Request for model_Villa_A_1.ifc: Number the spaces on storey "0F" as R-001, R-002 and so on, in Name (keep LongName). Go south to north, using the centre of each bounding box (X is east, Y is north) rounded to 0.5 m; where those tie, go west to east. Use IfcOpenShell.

First a look at what the model holds.

```python
import ifcopenshell
import ifcopenshell.util.element
import ifcopenshell.util.placement

model = ifcopenshell.open("model_Villa_A_1.ifc")
print(model.schema)
storey = next(s for s in model.by_type("IfcBuildingStorey") if s.Name == "0F")
spaces = [e for e in ifcopenshell.util.element.get_decomposition(storey) if e.is_a("IfcSpace")]
for e in sorted(spaces, key=lambda e: e.id()):
    origin = ifcopenshell.util.placement.get_local_placement(e.ObjectPlacement)[:3, 3]
    print(e.id(), e.Name, e.LongName, origin.round(2) + 0.0, sep=" | ")
```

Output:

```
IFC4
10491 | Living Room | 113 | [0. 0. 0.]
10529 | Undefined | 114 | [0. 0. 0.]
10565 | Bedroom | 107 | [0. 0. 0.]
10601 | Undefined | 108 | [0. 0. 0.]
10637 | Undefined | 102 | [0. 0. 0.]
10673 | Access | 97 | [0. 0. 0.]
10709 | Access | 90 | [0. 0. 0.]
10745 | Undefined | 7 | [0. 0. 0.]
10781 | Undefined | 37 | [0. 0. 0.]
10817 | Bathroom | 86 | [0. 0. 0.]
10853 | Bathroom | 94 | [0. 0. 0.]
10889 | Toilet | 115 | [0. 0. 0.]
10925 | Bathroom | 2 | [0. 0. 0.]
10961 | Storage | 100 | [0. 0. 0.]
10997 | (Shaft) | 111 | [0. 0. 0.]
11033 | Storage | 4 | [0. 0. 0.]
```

```python
import ifcopenshell
import ifcopenshell.geom
import ifcopenshell.util.element
import ifcopenshell.util.shape

model = ifcopenshell.open("model_Villa_A_1.ifc")
settings = ifcopenshell.geom.settings()
settings.set("use-world-coords", True)


def centre(element):
    shape = ifcopenshell.geom.create_shape(settings, element)
    return ifcopenshell.util.shape.get_bbox_centroid(shape.geometry)


storey = next(s for s in model.by_type("IfcBuildingStorey") if s.Name == "0F")
spaces = [e for e in ifcopenshell.util.element.get_decomposition(storey) if e.is_a("IfcSpace")]

# Insertion points can sit at a corner or the storey origin, so sort by the geometry (in metres).
centres = {e: centre(e) for e in spaces}
spaces.sort(key=lambda e: (round(centres[e][1] / 0.5), centres[e][0]))

for i, e in enumerate(spaces, start=1):
    number = f"R-0{i:02d}"
    e.Name = number
    print(e.id(), number)

model.write("model_Villa_A_1_rev.ifc")
```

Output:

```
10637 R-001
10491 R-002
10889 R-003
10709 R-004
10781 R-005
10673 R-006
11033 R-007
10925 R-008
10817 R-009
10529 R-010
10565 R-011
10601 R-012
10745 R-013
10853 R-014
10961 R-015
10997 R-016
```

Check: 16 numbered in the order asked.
